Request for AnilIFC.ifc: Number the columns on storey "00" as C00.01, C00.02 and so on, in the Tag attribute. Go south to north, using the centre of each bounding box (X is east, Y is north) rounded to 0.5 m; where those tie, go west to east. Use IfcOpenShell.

First a look at what the model holds.

```python
import ifcopenshell
import ifcopenshell.util.element
import ifcopenshell.util.placement

model = ifcopenshell.open("AnilIFC.ifc")
print(model.schema)
storey = next(s for s in model.by_type("IfcBuildingStorey") if s.Name == "00")
columns = [e for e in ifcopenshell.util.element.get_decomposition(storey) if e.is_a("IfcColumn")]
for e in sorted(columns, key=lambda e: e.id()):
    origin = ifcopenshell.util.placement.get_local_placement(e.ObjectPlacement)[:3, 3]
    print(e.id(), e.Tag, e.Name, origin.round(2) + 0.0, sep=" | ")
```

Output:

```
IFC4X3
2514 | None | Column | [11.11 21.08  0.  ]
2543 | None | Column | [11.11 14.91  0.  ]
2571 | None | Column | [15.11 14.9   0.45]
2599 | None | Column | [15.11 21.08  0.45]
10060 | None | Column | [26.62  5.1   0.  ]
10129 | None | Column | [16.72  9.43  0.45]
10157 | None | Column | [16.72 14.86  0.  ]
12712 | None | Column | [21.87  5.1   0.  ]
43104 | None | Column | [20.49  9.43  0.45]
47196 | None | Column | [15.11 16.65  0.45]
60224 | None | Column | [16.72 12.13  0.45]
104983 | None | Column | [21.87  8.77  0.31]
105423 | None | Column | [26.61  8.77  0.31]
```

```python
import ifcopenshell
import ifcopenshell.geom
import ifcopenshell.util.element
import ifcopenshell.util.shape

model = ifcopenshell.open("AnilIFC.ifc")
settings = ifcopenshell.geom.settings()
settings.set("use-world-coords", True)


def centre(element):
    shape = ifcopenshell.geom.create_shape(settings, element)
    return ifcopenshell.util.shape.get_bbox_centroid(shape.geometry)


storey = next(s for s in model.by_type("IfcBuildingStorey") if s.Name == "00")
columns = [e for e in ifcopenshell.util.element.get_decomposition(storey) if e.is_a("IfcColumn")]

# Insertion points can sit at a corner or the storey origin, so sort by the geometry (in metres).
centres = {e: centre(e) for e in columns}
columns.sort(key=lambda e: (round(centres[e][1] / 0.5), centres[e][0]))

for i, e in enumerate(columns, start=1):
    number = f"C00.{i:02d}"
    e.Tag = number
    print(e.id(), number)

model.write("AnilIFC_v2.ifc")
```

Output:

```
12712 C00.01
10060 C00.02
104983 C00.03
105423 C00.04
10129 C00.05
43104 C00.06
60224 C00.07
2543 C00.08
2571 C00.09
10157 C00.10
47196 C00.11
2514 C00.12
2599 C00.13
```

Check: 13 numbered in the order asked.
